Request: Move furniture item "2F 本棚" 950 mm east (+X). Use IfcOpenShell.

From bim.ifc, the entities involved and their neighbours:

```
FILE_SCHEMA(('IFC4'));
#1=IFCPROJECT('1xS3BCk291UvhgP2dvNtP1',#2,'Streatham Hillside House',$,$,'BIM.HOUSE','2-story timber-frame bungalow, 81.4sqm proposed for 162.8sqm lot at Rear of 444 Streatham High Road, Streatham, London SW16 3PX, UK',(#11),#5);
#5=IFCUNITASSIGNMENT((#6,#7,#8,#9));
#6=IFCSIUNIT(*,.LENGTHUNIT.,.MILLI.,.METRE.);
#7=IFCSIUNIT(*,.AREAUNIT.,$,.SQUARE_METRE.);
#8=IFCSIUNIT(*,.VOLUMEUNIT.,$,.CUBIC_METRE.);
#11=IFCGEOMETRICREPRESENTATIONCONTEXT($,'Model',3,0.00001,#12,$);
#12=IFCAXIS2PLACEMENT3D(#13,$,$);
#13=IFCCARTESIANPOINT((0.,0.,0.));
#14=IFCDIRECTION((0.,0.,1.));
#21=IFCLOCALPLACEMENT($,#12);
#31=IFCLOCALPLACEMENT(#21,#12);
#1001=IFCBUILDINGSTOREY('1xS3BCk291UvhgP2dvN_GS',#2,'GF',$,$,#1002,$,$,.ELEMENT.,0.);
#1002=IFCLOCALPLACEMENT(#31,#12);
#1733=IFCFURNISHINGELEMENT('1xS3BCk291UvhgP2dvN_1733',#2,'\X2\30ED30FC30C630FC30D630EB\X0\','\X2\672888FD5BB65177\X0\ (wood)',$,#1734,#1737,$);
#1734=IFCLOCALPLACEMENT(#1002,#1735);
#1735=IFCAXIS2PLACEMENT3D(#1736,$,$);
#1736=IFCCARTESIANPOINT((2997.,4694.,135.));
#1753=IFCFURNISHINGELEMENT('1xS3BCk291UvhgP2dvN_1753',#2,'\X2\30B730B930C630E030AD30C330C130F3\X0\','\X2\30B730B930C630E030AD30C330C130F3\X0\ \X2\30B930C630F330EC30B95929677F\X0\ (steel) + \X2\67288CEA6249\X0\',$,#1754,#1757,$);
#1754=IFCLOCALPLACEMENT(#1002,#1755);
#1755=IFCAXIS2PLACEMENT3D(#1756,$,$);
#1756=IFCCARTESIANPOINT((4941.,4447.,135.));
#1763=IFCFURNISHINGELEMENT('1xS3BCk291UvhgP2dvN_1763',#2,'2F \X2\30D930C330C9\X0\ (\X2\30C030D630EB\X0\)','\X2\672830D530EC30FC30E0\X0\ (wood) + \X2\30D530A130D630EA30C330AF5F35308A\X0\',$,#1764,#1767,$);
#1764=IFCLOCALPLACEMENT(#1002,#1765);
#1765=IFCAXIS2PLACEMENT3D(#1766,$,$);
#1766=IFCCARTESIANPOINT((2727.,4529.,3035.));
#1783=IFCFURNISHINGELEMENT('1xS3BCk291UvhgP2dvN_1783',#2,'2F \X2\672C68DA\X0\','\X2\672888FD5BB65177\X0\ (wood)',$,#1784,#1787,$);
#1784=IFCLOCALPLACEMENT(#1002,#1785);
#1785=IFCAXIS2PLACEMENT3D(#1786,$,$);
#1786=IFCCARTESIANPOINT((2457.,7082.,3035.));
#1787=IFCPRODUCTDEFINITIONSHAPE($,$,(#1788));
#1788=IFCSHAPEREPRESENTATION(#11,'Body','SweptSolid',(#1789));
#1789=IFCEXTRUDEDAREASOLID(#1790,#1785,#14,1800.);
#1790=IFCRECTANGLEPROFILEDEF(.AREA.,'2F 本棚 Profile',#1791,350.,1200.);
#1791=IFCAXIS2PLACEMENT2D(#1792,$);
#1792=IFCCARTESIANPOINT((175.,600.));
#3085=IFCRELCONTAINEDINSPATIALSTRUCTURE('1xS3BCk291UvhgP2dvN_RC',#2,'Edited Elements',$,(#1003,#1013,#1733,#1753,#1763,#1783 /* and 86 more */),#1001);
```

```python
import ifcopenshell
import ifcopenshell.api.geometry
import ifcopenshell.util.placement
import ifcopenshell.util.unit

model = ifcopenshell.open("bim.ifc")
unit_scale = ifcopenshell.util.unit.calculate_unit_scale(model)

item = model.by_guid("1xS3BCk291UvhgP2dvN_1783")
matrix = ifcopenshell.util.placement.get_local_placement(item.ObjectPlacement)
matrix[0, 3] += 0.95 / unit_scale
ifcopenshell.api.geometry.edit_object_placement(model, product=item, matrix=matrix, is_si=False)

print(ifcopenshell.util.placement.get_local_placement(item.ObjectPlacement).round(3) + 0.0)

model.write("bim_updated.ifc")
```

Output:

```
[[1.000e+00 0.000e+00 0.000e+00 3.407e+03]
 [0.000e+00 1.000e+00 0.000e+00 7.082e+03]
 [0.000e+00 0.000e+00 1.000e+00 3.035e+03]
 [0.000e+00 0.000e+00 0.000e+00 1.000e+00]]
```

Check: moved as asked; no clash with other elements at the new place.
